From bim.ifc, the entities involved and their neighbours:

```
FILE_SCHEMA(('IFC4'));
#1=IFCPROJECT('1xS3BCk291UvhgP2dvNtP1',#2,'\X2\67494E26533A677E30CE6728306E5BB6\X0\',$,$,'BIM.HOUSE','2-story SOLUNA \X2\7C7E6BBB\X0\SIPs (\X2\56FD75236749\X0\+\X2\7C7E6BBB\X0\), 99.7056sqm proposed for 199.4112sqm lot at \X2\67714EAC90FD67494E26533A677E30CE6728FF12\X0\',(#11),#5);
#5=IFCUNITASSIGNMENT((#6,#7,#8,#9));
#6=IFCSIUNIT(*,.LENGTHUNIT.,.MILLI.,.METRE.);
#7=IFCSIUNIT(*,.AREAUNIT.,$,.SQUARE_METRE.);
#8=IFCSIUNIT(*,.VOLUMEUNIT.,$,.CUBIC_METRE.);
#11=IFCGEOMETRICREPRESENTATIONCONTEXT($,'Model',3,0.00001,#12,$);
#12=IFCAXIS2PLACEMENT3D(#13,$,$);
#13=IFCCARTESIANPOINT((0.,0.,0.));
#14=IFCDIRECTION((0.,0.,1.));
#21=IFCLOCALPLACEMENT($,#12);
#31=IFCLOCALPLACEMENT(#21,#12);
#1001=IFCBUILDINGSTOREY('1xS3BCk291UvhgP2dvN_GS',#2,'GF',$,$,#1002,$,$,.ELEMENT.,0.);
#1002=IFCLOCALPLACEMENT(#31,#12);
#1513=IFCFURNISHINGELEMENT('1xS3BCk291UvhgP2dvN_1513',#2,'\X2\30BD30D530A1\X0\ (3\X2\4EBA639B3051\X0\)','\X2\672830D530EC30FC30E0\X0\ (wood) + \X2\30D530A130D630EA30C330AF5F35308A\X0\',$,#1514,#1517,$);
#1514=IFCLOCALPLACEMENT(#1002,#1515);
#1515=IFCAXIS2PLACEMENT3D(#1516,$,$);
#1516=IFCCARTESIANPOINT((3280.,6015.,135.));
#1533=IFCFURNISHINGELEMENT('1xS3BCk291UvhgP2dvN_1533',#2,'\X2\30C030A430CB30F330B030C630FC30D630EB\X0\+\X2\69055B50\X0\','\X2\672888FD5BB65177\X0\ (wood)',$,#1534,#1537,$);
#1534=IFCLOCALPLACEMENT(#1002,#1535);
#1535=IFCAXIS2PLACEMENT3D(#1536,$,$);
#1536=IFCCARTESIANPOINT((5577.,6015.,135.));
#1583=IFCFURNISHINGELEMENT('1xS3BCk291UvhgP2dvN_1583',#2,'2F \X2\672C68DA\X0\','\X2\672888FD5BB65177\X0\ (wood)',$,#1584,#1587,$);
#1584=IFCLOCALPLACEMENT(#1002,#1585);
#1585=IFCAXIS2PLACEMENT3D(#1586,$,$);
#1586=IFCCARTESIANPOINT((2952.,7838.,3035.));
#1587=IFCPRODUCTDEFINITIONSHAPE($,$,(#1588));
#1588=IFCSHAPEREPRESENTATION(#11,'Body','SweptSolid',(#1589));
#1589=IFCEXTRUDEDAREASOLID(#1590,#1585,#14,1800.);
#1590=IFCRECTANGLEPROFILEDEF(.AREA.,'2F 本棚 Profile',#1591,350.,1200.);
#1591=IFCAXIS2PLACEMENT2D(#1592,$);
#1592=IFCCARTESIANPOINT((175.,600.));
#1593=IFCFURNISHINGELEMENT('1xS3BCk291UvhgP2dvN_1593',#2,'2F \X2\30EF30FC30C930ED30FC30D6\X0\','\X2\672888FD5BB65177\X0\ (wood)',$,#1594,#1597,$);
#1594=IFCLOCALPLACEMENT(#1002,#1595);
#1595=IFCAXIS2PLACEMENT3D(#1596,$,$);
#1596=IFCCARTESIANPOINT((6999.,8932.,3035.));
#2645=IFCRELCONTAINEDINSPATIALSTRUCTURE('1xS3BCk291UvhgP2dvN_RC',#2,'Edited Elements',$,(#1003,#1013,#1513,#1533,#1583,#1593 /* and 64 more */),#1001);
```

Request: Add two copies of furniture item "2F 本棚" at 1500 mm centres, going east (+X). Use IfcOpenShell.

```python
import numpy as np
import ifcopenshell
import ifcopenshell.api.geometry
import ifcopenshell.api.root
import ifcopenshell.util.element
import ifcopenshell.util.placement

model = ifcopenshell.open("bim.ifc")


def reuse_history(source, copy):
    """copy_class also copies each property set's owner history, people and application; keep the originals."""
    for rel in copy.IsDefinedBy:
        if rel.is_a("IfcRelDefinesByProperties") and (history := rel.RelatingPropertyDefinition.OwnerHistory):
            rel.RelatingPropertyDefinition.OwnerHistory = source.OwnerHistory
            ifcopenshell.util.element.remove_deep2(model, history)


source = model.by_guid("1xS3BCk291UvhgP2dvN_1583")
base = ifcopenshell.util.placement.get_local_placement(source.ObjectPlacement)
step = np.array([1.0, 0.0, 0.0]) * 1500.0

for i in range(1, 3):
    copy = ifcopenshell.api.root.copy_class(model, product=source)
    copy.Representation = ifcopenshell.util.element.copy_deep(
        model, source.Representation, exclude=["IfcGeometricRepresentationContext", "IfcRepresentationMap"]
    )
    reuse_history(source, copy)
    matrix = base.copy()
    matrix[:3, 3] += i * step
    print("added at", matrix[:3, 3].round(3) + 0.0)
    ifcopenshell.api.geometry.edit_object_placement(model, product=copy, matrix=matrix, is_si=False)

model.write("bim_v2.ifc")
```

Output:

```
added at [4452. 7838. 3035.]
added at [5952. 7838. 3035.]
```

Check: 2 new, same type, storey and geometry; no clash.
